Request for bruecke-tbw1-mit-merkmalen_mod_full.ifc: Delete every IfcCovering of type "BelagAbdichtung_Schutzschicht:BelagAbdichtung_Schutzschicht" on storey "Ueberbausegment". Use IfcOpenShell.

First a look at what the model holds.

```python
import ifcopenshell
import ifcopenshell.util.element

model = ifcopenshell.open("bruecke-tbw1-mit-merkmalen_mod_full.ifc")
print(model.schema)
storey = next(s for s in model.by_type("IfcBuildingStorey") if s.Name == "Ueberbausegment")
coverings = [e for e in ifcopenshell.util.element.get_decomposition(storey) if e.is_a("IfcCovering")]
seen = {}
for e in coverings:
    element_type = ifcopenshell.util.element.get_type(e)
    name = element_type.Name if element_type not in (None, e) else None
    seen[name] = seen.get(name, 0) + 1
for name, count in sorted(seen.items(), key=str):
    print(count, "x", name)
```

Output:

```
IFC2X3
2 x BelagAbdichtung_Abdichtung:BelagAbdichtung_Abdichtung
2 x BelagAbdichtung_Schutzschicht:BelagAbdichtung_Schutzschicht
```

```python
import ifcopenshell
import ifcopenshell.api.root
import ifcopenshell.util.element

model = ifcopenshell.open("bruecke-tbw1-mit-merkmalen_mod_full.ifc")

storey = next(s for s in model.by_type("IfcBuildingStorey") if s.Name == "Ueberbausegment")
coverings = [e for e in ifcopenshell.util.element.get_decomposition(storey) if e.is_a("IfcCovering")]
targets = [e for e in coverings if (t := ifcopenshell.util.element.get_type(e)) not in (None, e) and t.Name == "BelagAbdichtung_Schutzschicht:BelagAbdichtung_Schutzschicht"]

for e in targets:
    ifcopenshell.api.root.remove_product(model, product=e)
print(len(targets), "removed")

model.write("bruecke-tbw1-mit-merkmalen_mod_full-out.ifc")
```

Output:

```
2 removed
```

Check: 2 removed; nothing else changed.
